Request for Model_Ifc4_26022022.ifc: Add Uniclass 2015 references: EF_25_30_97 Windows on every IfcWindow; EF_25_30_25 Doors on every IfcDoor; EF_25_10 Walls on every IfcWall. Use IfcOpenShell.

First a look at what the model holds.

```python
import ifcopenshell

model = ifcopenshell.open("Model_Ifc4_26022022.ifc")
print(model.schema)
print("classifications:", [c.Name for c in model.by_type("IfcClassification")])
for ifc_class in ("IfcDoor", "IfcRoof", "IfcStair", "IfcWall", "IfcWindow"):
    print(ifc_class, len(model.by_type(ifc_class)))
```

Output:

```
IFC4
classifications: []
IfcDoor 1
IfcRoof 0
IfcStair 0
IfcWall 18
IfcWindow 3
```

```python
import ifcopenshell
import ifcopenshell.api.classification

model = ifcopenshell.open("Model_Ifc4_26022022.ifc")

system = ifcopenshell.api.classification.add_classification(model, classification="Uniclass 2015")

codes = {
    "IfcWindow": ("EF_25_30_97", "Windows"),
    "IfcDoor": ("EF_25_30_25", "Doors"),
    "IfcWall": ("EF_25_10", "Walls"),
}
for ifc_class, (code, name) in codes.items():
    products = model.by_type(ifc_class)
    ifcopenshell.api.classification.add_reference(
        model, products=products, classification=system, identification=code, name=name
    )
    print(code, len(products))

model.write("Model_Ifc4_26022022_edited.ifc")
```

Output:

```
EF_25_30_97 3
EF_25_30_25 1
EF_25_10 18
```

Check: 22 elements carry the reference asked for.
